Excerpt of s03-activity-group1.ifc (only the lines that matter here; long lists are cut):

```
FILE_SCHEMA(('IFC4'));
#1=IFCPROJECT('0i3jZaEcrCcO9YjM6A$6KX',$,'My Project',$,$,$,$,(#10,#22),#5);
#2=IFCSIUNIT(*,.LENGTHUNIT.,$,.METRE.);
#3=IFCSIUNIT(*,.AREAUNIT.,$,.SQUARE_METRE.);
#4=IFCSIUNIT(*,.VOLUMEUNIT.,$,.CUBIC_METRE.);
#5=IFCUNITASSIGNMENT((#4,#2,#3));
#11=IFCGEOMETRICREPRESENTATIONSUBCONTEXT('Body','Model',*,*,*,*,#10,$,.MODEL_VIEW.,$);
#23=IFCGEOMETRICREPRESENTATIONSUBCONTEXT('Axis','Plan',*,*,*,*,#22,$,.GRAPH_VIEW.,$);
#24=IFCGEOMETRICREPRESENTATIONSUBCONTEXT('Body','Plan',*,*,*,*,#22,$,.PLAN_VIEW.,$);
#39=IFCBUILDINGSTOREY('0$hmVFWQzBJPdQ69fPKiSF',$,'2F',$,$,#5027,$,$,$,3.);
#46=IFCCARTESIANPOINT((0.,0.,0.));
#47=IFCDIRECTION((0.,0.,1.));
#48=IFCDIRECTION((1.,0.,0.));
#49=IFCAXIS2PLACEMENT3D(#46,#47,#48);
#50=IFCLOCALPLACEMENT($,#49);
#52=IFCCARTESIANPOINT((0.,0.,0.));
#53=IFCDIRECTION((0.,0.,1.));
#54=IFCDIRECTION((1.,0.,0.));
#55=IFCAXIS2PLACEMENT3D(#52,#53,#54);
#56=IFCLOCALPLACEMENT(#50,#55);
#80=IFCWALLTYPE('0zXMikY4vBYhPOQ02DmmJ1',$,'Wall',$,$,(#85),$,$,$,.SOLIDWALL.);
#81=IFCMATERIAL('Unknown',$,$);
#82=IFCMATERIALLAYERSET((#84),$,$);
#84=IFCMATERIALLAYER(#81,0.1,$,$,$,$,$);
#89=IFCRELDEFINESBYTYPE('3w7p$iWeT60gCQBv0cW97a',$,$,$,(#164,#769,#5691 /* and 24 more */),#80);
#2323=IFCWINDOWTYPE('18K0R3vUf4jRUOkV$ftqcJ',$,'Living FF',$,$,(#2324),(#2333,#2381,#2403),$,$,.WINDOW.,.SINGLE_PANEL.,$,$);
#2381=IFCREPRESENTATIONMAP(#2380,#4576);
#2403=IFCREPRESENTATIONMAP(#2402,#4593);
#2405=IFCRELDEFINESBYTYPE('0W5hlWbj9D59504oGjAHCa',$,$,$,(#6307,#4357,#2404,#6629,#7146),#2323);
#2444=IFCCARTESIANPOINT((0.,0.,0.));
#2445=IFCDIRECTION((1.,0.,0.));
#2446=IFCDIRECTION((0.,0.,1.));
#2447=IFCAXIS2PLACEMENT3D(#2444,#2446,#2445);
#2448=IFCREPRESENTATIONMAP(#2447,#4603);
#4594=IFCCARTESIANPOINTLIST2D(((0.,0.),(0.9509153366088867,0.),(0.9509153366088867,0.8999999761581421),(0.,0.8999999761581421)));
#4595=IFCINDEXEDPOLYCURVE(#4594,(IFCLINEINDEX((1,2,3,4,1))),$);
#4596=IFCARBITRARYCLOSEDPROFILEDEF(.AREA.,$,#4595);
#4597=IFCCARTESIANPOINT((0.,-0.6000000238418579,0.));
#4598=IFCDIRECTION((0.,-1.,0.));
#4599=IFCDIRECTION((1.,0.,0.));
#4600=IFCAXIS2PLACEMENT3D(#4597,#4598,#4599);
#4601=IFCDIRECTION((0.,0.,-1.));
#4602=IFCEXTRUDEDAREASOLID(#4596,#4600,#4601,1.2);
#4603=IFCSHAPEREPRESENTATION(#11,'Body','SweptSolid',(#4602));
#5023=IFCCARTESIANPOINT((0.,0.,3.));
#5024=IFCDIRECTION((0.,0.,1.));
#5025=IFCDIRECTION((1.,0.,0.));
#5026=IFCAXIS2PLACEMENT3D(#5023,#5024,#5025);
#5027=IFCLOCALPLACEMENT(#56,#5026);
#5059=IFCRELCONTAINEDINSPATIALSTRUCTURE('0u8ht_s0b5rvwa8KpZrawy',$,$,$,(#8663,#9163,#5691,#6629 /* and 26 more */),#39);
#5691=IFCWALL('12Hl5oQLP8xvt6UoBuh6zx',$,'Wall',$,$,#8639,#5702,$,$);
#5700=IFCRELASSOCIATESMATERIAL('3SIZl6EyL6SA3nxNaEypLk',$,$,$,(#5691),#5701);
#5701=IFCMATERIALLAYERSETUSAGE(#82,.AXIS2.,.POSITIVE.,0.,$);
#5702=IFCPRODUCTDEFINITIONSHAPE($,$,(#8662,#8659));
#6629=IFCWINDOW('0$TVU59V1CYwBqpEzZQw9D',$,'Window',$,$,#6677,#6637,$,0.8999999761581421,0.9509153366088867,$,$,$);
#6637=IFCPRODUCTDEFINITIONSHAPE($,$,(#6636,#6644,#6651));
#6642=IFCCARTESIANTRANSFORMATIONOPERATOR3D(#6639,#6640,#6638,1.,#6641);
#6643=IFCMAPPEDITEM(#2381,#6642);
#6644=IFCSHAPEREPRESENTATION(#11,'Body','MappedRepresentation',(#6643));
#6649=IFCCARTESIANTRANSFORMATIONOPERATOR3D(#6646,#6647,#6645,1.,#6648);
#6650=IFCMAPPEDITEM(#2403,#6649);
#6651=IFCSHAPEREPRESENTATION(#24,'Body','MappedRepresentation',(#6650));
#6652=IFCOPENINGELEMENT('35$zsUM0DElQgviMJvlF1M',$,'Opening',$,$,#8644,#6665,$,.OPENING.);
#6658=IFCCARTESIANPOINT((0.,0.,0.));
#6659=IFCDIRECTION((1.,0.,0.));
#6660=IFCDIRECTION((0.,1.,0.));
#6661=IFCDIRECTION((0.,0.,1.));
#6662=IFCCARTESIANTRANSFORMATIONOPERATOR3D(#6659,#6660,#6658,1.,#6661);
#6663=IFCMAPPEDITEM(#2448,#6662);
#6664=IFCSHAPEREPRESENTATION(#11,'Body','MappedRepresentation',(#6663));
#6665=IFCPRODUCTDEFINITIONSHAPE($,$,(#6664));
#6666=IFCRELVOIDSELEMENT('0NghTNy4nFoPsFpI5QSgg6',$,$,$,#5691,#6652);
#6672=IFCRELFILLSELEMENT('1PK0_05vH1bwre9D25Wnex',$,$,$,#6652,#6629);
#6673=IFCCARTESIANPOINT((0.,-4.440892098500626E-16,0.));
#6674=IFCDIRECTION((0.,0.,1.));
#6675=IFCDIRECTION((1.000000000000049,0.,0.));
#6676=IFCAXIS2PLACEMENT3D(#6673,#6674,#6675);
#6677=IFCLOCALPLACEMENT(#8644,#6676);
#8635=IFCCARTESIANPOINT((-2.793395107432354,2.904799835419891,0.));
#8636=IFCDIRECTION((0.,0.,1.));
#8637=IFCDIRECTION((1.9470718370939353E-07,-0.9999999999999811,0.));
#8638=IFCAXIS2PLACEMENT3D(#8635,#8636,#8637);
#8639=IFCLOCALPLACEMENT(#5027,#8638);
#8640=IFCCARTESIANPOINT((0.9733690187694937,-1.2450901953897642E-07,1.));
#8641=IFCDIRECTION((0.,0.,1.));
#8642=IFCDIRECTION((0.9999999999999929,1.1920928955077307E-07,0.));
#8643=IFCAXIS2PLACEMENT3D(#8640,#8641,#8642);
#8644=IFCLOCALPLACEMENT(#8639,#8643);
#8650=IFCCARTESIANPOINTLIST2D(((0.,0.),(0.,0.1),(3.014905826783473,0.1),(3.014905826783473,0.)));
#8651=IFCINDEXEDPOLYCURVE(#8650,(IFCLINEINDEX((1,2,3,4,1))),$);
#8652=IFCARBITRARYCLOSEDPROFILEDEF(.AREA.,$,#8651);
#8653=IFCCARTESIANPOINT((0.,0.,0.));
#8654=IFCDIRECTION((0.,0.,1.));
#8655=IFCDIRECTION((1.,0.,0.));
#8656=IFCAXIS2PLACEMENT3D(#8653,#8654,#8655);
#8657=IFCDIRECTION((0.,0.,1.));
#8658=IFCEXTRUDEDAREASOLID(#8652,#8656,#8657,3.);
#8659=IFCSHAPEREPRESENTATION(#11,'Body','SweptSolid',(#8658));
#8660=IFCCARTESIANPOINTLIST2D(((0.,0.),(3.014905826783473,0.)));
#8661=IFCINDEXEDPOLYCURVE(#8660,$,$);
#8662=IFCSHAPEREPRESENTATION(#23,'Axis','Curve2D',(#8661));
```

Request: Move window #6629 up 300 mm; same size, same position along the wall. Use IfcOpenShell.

```python
import numpy as np
import ifcopenshell
import ifcopenshell.api.geometry
import ifcopenshell.util.placement
import ifcopenshell.util.unit

model = ifcopenshell.open("s03-activity-group1.ifc")
unit_scale = ifcopenshell.util.unit.calculate_unit_scale(model)

window = model.by_guid("0$TVU59V1CYwBqpEzZQw9D")
opening = window.FillsVoids[0].RelatingOpeningElement
dz = 0.3 / unit_scale

shift = np.array([0.0, 0.0, dz])
# The window is placed relative to its opening, so it follows when the opening moves.
matrix = ifcopenshell.util.placement.get_local_placement(opening.ObjectPlacement)
matrix[:3, 3] += shift
ifcopenshell.api.geometry.edit_object_placement(
    model, product=opening, matrix=matrix, is_si=False, should_transform_children=True
)

print(f"moved by {dz * unit_scale:+.3f} m")

model.write("s03-activity-group1_updated.ifc")
```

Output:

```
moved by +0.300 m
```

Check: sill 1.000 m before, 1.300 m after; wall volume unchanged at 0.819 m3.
